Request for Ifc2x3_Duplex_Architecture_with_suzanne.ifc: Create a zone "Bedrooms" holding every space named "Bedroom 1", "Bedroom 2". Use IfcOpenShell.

First a look at what the model holds.

```python
import ifcopenshell

model = ifcopenshell.open("Ifc2x3_Duplex_Architecture_with_suzanne.ifc")
print(model.schema)
seen = {}
for space in model.by_type("IfcSpace"):
    seen[space.LongName] = seen.get(space.LongName, 0) + 1
for name, count in sorted(seen.items(), key=str):
    print(count, "x", name)
print("zones:", [z.Name for z in model.by_type("IfcZone")][:20])
```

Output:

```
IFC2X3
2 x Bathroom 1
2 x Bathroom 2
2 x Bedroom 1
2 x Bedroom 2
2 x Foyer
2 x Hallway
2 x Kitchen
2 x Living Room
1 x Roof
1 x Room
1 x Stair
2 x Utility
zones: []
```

```python
import ifcopenshell
import ifcopenshell.api.group
import ifcopenshell.api.root

model = ifcopenshell.open("Ifc2x3_Duplex_Architecture_with_suzanne.ifc")

names = {"Bedroom 1", "Bedroom 2"}
spaces = [s for s in model.by_type("IfcSpace") if s.LongName in names]

zone = ifcopenshell.api.root.create_entity(model, ifc_class="IfcZone", name="Bedrooms")
ifcopenshell.api.group.assign_group(model, products=spaces, group=zone)
print(len(spaces), "spaces in", zone.Name)

model.write("Ifc2x3_Duplex_Architecture_with_suzanne_edited.ifc")
```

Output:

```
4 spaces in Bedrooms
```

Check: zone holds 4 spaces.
